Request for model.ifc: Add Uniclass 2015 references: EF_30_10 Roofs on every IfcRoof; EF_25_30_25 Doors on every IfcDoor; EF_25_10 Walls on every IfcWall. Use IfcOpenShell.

First a look at what the model holds.

```python
import ifcopenshell

model = ifcopenshell.open("model.ifc")
print(model.schema)
print("classifications:", [c.Name for c in model.by_type("IfcClassification")])
for ifc_class in ("IfcDoor", "IfcRoof", "IfcStair", "IfcWall", "IfcWindow"):
    print(ifc_class, len(model.by_type(ifc_class)))
```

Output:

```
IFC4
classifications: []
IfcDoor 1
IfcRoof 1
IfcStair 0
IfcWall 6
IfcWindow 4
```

```python
import ifcopenshell
import ifcopenshell.api.classification

model = ifcopenshell.open("model.ifc")

system = ifcopenshell.api.classification.add_classification(model, classification="Uniclass 2015")

codes = {
    "IfcRoof": ("EF_30_10", "Roofs"),
    "IfcDoor": ("EF_25_30_25", "Doors"),
    "IfcWall": ("EF_25_10", "Walls"),
}
for ifc_class, (code, name) in codes.items():
    products = model.by_type(ifc_class)
    ifcopenshell.api.classification.add_reference(
        model, products=products, classification=system, identification=code, name=name
    )
    print(code, len(products))

model.write("model_edited.ifc")
```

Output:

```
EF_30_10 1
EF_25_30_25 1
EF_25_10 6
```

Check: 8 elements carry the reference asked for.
